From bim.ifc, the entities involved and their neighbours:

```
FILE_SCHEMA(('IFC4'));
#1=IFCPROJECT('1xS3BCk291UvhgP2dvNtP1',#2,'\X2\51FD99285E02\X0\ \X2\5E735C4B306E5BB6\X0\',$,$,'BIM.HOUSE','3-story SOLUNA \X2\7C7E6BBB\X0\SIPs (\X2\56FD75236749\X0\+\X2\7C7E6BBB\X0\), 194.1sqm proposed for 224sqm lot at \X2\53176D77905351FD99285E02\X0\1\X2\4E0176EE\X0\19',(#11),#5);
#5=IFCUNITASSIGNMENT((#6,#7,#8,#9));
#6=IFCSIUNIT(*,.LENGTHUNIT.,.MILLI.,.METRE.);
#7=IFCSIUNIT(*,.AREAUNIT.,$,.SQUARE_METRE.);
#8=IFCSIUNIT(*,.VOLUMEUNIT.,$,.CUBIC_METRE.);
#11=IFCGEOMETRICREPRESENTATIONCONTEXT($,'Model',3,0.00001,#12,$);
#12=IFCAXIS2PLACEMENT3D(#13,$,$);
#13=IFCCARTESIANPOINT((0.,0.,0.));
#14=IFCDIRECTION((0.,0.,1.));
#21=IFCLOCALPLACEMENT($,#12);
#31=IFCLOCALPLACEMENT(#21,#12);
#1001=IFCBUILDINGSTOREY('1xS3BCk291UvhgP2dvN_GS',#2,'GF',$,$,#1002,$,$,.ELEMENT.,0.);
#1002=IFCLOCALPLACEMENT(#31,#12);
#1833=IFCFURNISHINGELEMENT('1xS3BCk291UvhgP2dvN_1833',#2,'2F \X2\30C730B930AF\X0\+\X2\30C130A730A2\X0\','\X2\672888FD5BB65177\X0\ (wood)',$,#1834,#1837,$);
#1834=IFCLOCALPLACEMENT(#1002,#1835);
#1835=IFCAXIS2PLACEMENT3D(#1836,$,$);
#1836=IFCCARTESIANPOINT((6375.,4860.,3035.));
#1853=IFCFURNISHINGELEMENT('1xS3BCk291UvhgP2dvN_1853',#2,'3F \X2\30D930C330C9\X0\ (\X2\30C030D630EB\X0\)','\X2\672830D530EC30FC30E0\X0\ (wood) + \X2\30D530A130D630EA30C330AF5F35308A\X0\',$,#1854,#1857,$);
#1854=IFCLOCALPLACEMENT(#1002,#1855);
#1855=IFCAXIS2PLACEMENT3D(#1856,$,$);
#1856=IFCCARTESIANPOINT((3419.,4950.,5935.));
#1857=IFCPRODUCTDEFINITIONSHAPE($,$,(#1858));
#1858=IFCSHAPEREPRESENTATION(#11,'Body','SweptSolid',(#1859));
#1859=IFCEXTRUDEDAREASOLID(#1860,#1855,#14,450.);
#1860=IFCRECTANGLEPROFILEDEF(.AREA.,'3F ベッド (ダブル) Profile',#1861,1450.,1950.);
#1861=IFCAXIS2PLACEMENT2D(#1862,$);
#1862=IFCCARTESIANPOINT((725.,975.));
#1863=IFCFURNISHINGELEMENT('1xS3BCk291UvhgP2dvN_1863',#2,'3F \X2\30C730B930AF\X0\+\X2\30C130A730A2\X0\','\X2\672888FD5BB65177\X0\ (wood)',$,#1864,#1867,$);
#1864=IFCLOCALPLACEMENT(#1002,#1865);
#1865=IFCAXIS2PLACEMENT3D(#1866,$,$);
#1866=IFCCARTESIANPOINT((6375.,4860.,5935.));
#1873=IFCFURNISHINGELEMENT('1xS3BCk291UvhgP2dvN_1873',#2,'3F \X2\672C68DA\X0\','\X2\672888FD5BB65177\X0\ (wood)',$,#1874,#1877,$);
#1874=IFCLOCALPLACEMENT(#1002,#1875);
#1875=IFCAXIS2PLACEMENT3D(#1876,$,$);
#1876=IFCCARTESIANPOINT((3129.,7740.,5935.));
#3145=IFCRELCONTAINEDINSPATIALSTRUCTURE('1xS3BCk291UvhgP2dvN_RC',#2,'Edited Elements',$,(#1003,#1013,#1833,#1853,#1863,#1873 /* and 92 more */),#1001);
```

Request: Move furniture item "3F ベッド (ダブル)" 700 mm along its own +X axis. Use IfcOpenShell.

```python
import ifcopenshell
import ifcopenshell.api.geometry
import ifcopenshell.util.placement
import ifcopenshell.util.unit

model = ifcopenshell.open("bim.ifc")
unit_scale = ifcopenshell.util.unit.calculate_unit_scale(model)

item = model.by_id(1853)
matrix = ifcopenshell.util.placement.get_local_placement(item.ObjectPlacement)
matrix[:3, 3] += matrix[:3, 0] * 0.7 / unit_scale
ifcopenshell.api.geometry.edit_object_placement(model, product=item, matrix=matrix, is_si=False)

print(ifcopenshell.util.placement.get_local_placement(item.ObjectPlacement).round(3) + 0.0)

model.write("bim_rev.ifc")
```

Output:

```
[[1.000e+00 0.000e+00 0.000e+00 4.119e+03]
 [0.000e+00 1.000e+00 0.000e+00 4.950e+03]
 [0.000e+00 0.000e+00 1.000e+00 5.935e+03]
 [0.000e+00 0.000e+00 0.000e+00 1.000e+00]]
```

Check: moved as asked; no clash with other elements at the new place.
